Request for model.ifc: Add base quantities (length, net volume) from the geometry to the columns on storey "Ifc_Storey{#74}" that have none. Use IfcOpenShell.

First a look at what the model holds.

```python
import ifcopenshell
import ifcopenshell.util.element
import ifcopenshell.util.unit

model = ifcopenshell.open("model.ifc")
print(model.schema)
for unit_type in ("LENGTHUNIT", "AREAUNIT", "VOLUMEUNIT"):
    print(unit_type, ifcopenshell.util.unit.calculate_unit_scale(model, unit_type))
storey = next(s for s in model.by_type("IfcBuildingStorey") if s.Name == "Ifc_Storey{#74}")
columns = [e for e in ifcopenshell.util.element.get_decomposition(storey) if e.is_a("IfcColumn")]
for e in sorted(columns, key=lambda e: e.id()):
    print(e.id(), e.is_a(), e.Name, list(ifcopenshell.util.element.get_psets(e, qtos_only=True)), sep=" | ")
```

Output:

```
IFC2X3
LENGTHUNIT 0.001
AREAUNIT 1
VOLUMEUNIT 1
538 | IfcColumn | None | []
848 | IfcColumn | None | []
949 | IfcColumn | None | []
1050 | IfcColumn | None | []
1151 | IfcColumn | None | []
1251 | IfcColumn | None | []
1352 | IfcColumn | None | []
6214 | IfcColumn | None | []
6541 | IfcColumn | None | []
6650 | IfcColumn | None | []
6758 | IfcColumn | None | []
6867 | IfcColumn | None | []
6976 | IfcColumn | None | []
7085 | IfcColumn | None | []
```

```python
import ifcopenshell
import ifcopenshell.api.pset
import ifcopenshell.geom
import ifcopenshell.util.element
import ifcopenshell.util.shape
import ifcopenshell.util.unit

model = ifcopenshell.open("model.ifc")
unit_scale = ifcopenshell.util.unit.calculate_unit_scale(model)
volume_scale = ifcopenshell.util.unit.calculate_unit_scale(model, "VOLUMEUNIT")
settings = ifcopenshell.geom.settings()

storey = next(s for s in model.by_type("IfcBuildingStorey") if s.Name == "Ifc_Storey{#74}")
columns = [e for e in ifcopenshell.util.element.get_decomposition(storey) if e.is_a("IfcColumn")]

for e in sorted(columns, key=lambda e: e.id()):
    if ifcopenshell.util.element.get_psets(e, qtos_only=True, should_inherit=False):
        continue
    # Geometry comes back in metres, in the element's own axes.
    shape = ifcopenshell.geom.create_shape(settings, e)
    values = {
        "Length": ifcopenshell.util.shape.get_z(shape.geometry) / unit_scale,
        "NetVolume": ifcopenshell.util.shape.get_volume(shape.geometry) / volume_scale,
    }
    qto = ifcopenshell.api.pset.add_qto(model, product=e, name="BaseQuantities")
    ifcopenshell.api.pset.edit_qto(model, qto=qto, properties=values)
    print(e.id(), {k: round(v, 3) for k, v in values.items()})

model.write("model_edited.ifc")
```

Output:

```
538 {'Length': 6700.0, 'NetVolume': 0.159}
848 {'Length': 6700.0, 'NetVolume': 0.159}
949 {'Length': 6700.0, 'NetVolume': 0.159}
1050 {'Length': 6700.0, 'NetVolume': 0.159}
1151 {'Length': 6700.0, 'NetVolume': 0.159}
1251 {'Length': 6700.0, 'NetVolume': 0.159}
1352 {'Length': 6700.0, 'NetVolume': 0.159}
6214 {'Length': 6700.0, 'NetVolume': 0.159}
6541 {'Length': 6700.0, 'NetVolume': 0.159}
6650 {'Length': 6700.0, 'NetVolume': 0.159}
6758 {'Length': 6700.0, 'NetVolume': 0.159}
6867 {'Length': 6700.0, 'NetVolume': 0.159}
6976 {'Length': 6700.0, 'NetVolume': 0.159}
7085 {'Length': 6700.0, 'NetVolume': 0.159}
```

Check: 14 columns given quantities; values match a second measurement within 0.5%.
